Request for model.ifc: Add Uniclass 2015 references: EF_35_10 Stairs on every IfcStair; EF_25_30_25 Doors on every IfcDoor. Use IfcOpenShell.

First a look at what the model holds.

```python
import ifcopenshell

model = ifcopenshell.open("model.ifc")
print(model.schema)
print("classifications:", [c.Name for c in model.by_type("IfcClassification")])
for ifc_class in ("IfcDoor", "IfcRoof", "IfcStair", "IfcWall", "IfcWindow"):
    print(ifc_class, len(model.by_type(ifc_class)))
```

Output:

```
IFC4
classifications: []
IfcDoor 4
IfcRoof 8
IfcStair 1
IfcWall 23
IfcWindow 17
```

```python
import ifcopenshell
import ifcopenshell.api.classification

model = ifcopenshell.open("model.ifc")

system = ifcopenshell.api.classification.add_classification(model, classification="Uniclass 2015")

codes = {
    "IfcStair": ("EF_35_10", "Stairs"),
    "IfcDoor": ("EF_25_30_25", "Doors"),
}
for ifc_class, (code, name) in codes.items():
    products = model.by_type(ifc_class)
    ifcopenshell.api.classification.add_reference(
        model, products=products, classification=system, identification=code, name=name
    )
    print(code, len(products))

model.write("model-out.ifc")
```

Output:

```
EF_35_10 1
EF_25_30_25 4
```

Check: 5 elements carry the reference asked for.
